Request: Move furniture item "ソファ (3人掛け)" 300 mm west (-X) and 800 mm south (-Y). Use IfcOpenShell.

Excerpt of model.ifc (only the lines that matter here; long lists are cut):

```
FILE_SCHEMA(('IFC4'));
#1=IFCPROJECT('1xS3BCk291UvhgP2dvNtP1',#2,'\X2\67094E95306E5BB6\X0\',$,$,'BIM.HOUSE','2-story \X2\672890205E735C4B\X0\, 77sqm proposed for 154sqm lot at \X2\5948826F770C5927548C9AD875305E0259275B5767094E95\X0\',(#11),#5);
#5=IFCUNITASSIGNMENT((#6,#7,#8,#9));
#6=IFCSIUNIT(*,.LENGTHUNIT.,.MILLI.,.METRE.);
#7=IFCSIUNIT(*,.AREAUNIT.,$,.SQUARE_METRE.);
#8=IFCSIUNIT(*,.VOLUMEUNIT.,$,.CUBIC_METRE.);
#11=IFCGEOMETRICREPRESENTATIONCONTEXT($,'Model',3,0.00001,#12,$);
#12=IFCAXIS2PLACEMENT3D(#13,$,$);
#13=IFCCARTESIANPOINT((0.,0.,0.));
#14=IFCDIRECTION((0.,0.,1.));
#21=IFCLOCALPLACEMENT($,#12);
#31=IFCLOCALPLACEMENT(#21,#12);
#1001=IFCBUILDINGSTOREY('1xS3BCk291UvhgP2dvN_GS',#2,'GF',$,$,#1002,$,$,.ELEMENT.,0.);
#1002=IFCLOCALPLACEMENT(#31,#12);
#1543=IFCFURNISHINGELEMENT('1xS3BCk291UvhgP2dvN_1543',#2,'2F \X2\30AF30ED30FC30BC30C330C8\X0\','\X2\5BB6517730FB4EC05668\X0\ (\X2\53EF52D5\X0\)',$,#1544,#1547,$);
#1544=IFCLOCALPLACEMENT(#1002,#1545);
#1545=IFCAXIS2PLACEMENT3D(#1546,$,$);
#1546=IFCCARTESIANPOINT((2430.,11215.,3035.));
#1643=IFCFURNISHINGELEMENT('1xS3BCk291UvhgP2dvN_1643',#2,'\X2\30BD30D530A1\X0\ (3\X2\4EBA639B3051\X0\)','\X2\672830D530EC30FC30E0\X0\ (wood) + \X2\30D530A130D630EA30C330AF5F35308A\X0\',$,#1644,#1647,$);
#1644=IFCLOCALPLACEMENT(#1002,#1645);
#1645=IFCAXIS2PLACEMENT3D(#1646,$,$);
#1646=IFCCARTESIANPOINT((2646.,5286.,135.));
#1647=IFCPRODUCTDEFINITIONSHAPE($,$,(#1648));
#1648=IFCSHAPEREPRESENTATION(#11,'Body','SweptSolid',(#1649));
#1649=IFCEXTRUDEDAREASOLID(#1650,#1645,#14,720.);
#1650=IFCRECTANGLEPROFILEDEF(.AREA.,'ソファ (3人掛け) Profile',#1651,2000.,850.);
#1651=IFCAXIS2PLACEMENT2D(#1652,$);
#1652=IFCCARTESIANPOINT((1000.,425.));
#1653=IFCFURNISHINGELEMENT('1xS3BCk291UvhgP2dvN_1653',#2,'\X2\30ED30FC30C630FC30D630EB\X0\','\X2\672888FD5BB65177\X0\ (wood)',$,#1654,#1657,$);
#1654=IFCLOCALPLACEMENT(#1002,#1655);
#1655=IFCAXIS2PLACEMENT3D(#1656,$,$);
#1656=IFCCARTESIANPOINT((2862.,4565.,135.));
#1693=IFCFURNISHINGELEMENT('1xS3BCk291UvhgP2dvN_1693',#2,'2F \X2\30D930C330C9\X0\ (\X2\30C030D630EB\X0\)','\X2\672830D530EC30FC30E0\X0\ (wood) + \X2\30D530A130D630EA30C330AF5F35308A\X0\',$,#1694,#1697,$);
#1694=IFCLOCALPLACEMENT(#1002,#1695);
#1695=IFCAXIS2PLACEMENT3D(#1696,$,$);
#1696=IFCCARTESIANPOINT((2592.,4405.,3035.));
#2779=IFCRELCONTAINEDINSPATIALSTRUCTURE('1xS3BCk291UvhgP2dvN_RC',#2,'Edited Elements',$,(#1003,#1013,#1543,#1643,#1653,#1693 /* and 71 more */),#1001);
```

```python
import ifcopenshell
import ifcopenshell.api.geometry
import ifcopenshell.util.placement

model = ifcopenshell.open("model.ifc")

item = model.by_guid("1xS3BCk291UvhgP2dvN_1643")
matrix = ifcopenshell.util.placement.get_local_placement(item.ObjectPlacement)
matrix[0, 3] -= 300.0
matrix[1, 3] -= 800.0
ifcopenshell.api.geometry.edit_object_placement(model, product=item, matrix=matrix, is_si=False)

print(ifcopenshell.util.placement.get_local_placement(item.ObjectPlacement).round(3) + 0.0)

model.write("model_edited.ifc")
```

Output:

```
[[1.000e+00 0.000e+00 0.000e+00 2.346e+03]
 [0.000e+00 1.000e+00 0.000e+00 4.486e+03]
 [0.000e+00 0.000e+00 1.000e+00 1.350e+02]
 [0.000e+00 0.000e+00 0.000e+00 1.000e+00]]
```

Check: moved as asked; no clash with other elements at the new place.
